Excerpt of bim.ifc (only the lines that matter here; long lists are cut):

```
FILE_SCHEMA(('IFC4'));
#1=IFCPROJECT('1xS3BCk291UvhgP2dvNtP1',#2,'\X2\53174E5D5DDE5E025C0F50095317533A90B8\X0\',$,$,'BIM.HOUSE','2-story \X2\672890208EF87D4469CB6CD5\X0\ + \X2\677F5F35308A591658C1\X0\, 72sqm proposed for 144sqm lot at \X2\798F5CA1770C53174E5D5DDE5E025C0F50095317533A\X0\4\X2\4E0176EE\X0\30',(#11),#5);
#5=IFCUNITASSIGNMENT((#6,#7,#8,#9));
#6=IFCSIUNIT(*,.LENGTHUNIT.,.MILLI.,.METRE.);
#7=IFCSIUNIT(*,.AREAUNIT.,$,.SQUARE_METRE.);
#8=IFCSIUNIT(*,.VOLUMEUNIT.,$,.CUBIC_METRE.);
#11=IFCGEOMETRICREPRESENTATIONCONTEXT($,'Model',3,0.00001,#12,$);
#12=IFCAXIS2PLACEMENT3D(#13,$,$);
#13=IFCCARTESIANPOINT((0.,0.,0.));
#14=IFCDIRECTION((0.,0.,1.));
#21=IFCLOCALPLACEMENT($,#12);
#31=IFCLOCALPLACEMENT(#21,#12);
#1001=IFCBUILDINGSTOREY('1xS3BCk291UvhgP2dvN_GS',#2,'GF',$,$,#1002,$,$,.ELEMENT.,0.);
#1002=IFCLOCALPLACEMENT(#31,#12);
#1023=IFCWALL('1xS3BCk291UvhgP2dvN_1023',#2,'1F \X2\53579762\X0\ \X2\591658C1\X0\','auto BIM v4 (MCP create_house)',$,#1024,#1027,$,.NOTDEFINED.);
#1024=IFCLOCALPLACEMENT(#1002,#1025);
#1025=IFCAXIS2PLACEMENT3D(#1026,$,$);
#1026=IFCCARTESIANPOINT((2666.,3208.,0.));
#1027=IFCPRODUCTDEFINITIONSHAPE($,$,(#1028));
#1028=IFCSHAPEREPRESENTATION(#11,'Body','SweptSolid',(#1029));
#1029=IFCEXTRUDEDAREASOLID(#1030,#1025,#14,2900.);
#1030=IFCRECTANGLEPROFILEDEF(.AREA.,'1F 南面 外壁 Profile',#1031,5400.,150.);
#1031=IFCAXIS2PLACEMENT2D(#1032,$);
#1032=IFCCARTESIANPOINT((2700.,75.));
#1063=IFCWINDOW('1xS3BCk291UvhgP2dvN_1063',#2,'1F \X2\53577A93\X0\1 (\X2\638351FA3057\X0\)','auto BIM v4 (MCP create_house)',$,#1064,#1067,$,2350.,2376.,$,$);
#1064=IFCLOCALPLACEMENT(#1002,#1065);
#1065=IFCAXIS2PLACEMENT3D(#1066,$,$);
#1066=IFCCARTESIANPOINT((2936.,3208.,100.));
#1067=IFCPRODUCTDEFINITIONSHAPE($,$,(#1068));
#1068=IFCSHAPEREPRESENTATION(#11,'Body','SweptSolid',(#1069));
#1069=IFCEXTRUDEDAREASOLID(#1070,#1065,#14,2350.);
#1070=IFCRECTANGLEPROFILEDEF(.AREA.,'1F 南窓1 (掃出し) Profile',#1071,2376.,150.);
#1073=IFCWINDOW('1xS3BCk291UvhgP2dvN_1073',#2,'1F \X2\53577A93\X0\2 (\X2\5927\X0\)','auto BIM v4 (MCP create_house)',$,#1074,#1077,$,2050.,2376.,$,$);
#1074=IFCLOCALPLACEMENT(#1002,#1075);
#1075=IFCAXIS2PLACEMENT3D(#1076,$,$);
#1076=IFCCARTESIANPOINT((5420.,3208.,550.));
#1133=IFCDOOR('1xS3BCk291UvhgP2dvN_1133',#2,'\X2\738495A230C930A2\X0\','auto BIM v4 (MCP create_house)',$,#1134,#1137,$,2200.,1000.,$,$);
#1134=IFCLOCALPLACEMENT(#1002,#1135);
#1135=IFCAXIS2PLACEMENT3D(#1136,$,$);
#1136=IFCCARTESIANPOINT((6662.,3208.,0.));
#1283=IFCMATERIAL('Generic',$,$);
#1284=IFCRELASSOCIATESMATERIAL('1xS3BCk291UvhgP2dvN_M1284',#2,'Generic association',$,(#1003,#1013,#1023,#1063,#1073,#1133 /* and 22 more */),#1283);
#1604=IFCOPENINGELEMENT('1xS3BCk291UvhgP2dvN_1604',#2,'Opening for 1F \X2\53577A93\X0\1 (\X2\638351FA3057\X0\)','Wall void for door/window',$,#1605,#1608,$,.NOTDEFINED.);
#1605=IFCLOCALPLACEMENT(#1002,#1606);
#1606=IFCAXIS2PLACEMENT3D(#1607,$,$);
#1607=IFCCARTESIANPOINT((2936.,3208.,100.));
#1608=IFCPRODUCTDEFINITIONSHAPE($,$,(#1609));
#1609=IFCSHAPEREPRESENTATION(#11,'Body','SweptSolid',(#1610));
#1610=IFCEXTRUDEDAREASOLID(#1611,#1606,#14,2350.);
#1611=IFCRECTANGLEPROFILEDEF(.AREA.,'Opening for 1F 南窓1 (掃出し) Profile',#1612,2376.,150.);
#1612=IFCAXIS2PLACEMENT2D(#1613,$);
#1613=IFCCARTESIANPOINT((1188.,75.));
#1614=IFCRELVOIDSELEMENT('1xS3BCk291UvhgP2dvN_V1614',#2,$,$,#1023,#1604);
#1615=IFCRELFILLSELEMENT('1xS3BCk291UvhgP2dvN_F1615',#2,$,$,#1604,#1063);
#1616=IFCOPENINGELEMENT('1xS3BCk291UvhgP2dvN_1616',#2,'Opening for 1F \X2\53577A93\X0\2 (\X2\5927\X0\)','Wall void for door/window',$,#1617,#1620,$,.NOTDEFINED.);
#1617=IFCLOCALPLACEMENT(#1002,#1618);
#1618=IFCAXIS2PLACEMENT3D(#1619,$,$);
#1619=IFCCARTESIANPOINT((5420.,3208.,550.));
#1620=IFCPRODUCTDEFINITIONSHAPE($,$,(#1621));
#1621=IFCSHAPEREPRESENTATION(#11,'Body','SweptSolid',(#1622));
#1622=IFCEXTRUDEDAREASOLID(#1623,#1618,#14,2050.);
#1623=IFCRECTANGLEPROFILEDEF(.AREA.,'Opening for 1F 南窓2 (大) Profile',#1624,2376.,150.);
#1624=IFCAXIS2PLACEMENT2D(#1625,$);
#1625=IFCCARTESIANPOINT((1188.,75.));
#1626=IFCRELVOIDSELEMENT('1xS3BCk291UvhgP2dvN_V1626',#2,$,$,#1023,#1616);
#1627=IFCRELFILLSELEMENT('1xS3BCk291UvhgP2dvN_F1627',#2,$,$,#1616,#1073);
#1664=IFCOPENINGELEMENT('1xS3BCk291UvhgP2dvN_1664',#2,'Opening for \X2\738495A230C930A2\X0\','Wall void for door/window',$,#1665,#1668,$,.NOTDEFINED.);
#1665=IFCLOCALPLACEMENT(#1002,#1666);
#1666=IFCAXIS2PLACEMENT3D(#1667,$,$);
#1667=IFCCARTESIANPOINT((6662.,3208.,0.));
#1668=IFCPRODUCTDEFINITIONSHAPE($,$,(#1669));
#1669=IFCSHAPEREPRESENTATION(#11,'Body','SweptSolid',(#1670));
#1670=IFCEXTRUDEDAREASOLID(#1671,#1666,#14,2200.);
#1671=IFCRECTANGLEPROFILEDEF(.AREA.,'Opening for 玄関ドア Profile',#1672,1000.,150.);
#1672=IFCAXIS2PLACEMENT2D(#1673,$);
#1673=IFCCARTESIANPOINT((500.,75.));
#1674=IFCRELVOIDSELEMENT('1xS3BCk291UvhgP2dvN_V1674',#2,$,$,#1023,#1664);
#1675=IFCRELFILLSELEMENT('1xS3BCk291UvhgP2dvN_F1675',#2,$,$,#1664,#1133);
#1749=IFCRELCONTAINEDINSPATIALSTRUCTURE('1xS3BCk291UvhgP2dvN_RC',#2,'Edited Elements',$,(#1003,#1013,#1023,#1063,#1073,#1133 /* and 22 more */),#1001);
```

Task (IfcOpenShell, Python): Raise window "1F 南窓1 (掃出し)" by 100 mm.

```python
import numpy as np
import ifcopenshell
import ifcopenshell.api.geometry
import ifcopenshell.util.placement
import ifcopenshell.util.unit

model = ifcopenshell.open("bim.ifc")
unit_scale = ifcopenshell.util.unit.calculate_unit_scale(model)

window = model.by_guid("1xS3BCk291UvhgP2dvN_1063")
opening = window.FillsVoids[0].RelatingOpeningElement
dz = 100.0

shift = np.array([0.0, 0.0, dz])
# The window is not placed relative to its opening, so move both.
for product in (opening, window):
    matrix = ifcopenshell.util.placement.get_local_placement(product.ObjectPlacement)
    matrix[:3, 3] += shift
    ifcopenshell.api.geometry.edit_object_placement(model, product=product, matrix=matrix, is_si=False)

print(f"moved by {dz * unit_scale:+.3f} m")

model.write("bim_rev.ifc")
```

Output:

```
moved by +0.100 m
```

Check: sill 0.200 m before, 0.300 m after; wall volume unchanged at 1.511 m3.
